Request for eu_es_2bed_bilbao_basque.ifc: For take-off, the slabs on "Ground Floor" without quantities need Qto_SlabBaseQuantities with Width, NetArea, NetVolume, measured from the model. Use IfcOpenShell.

First a look at what the model holds.

```python
import ifcopenshell
import ifcopenshell.util.element
import ifcopenshell.util.unit

model = ifcopenshell.open("eu_es_2bed_bilbao_basque.ifc")
print(model.schema)
for unit_type in ("LENGTHUNIT", "AREAUNIT", "VOLUMEUNIT"):
    print(unit_type, ifcopenshell.util.unit.calculate_unit_scale(model, unit_type))
storey = next(s for s in model.by_type("IfcBuildingStorey") if s.Name == "Ground Floor")
slabs = [e for e in ifcopenshell.util.element.get_decomposition(storey) if e.is_a("IfcSlab")]
for e in sorted(slabs, key=lambda e: e.id()):
    print(e.id(), e.is_a(), e.Name, list(ifcopenshell.util.element.get_psets(e, qtos_only=True)), sep=" | ")
```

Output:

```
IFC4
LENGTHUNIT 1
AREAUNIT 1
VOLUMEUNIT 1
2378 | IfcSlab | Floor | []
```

```python
import ifcopenshell
import ifcopenshell.api.pset
import ifcopenshell.geom
import ifcopenshell.util.element
import ifcopenshell.util.shape
import ifcopenshell.util.unit

model = ifcopenshell.open("eu_es_2bed_bilbao_basque.ifc")
unit_scale = ifcopenshell.util.unit.calculate_unit_scale(model)
area_scale = ifcopenshell.util.unit.calculate_unit_scale(model, "AREAUNIT")
volume_scale = ifcopenshell.util.unit.calculate_unit_scale(model, "VOLUMEUNIT")
settings = ifcopenshell.geom.settings()

storey = next(s for s in model.by_type("IfcBuildingStorey") if s.Name == "Ground Floor")
slabs = [e for e in ifcopenshell.util.element.get_decomposition(storey) if e.is_a("IfcSlab")]

for e in sorted(slabs, key=lambda e: e.id()):
    if ifcopenshell.util.element.get_psets(e, qtos_only=True, should_inherit=False):
        continue
    # Geometry comes back in metres, in the element's own axes.
    shape = ifcopenshell.geom.create_shape(settings, e)
    values = {
        "Width": ifcopenshell.util.shape.get_z(shape.geometry) / unit_scale,
        "NetArea": ifcopenshell.util.shape.get_footprint_area(shape.geometry) / area_scale,
        "NetVolume": ifcopenshell.util.shape.get_volume(shape.geometry) / volume_scale,
    }
    qto = ifcopenshell.api.pset.add_qto(model, product=e, name="Qto_SlabBaseQuantities")
    ifcopenshell.api.pset.edit_qto(model, qto=qto, properties=values)
    print(e.id(), {k: round(v, 3) for k, v in values.items()})

model.write("eu_es_2bed_bilbao_basque-out.ifc")
```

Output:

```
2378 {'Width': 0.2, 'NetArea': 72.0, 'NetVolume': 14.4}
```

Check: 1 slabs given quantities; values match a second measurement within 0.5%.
